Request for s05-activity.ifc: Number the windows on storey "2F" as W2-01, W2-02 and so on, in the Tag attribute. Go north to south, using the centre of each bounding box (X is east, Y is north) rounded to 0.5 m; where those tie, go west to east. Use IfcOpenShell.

First a look at what the model holds.

```python
import ifcopenshell
import ifcopenshell.util.element
import ifcopenshell.util.placement

model = ifcopenshell.open("s05-activity.ifc")
print(model.schema)
storey = next(s for s in model.by_type("IfcBuildingStorey") if s.Name == "2F")
windows = [e for e in ifcopenshell.util.element.get_decomposition(storey) if e.is_a("IfcWindow")]
for e in sorted(windows, key=lambda e: e.id()):
    origin = ifcopenshell.util.placement.get_local_placement(e.ObjectPlacement)[:3, 3]
    print(e.id(), e.Tag, e.Name, origin.round(2) + 0.0, sep=" | ")
```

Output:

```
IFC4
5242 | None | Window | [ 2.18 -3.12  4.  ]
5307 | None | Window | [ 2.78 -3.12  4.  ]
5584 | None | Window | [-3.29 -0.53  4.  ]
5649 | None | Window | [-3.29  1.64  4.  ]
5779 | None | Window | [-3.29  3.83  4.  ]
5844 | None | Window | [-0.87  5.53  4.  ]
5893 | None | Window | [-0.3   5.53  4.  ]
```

```python
import ifcopenshell
import ifcopenshell.geom
import ifcopenshell.util.element
import ifcopenshell.util.shape

model = ifcopenshell.open("s05-activity.ifc")
settings = ifcopenshell.geom.settings()
settings.set("use-world-coords", True)


def centre(element):
    shape = ifcopenshell.geom.create_shape(settings, element)
    return ifcopenshell.util.shape.get_bbox_centroid(shape.geometry)


storey = next(s for s in model.by_type("IfcBuildingStorey") if s.Name == "2F")
windows = [e for e in ifcopenshell.util.element.get_decomposition(storey) if e.is_a("IfcWindow")]

# Insertion points can sit at a corner or the storey origin, so sort by the geometry (in metres).
centres = {e: centre(e) for e in windows}
windows.sort(key=lambda e: (-round(centres[e][1] / 0.5), centres[e][0]))

for i, e in enumerate(windows, start=1):
    number = f"W2-{i:02d}"
    e.Tag = number
    print(e.id(), number)

model.write("s05-activity_rev.ifc")
```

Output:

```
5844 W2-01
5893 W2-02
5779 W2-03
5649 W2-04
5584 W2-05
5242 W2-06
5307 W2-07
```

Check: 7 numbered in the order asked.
